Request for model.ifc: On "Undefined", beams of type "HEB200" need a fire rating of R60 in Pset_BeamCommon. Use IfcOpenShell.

First a look at what the model holds.

```python
import ifcopenshell
import ifcopenshell.util.element

model = ifcopenshell.open("model.ifc")
print(model.schema)
storey = next(s for s in model.by_type("IfcBuildingStorey") if s.Name == "Undefined")
beams = [e for e in ifcopenshell.util.element.get_decomposition(storey) if e.is_a("IfcBeam")]
seen = {}
for e in beams:
    element_type = ifcopenshell.util.element.get_type(e)
    key = (element_type.Name if element_type != e and element_type else None, ifcopenshell.util.element.get_pset(e, "Pset_BeamCommon", "FireRating"))
    seen[key] = seen.get(key, 0) + 1
for (name, value), count in sorted(seen.items(), key=str):
    print(count, "x", name, "|", value)
```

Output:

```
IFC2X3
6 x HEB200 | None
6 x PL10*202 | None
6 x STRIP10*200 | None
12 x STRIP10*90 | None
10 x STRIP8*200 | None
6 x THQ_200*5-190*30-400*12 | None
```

```python
import ifcopenshell
import ifcopenshell.api.pset
import ifcopenshell.util.element

model = ifcopenshell.open("model.ifc")

storey = next(s for s in model.by_type("IfcBuildingStorey") if s.Name == "Undefined")
beams = [e for e in ifcopenshell.util.element.get_decomposition(storey) if e.is_a("IfcBeam")]

count = 0
for e in beams:
    element_type = ifcopenshell.util.element.get_type(e)
    if element_type in (None, e) or element_type.Name != "HEB200":
        continue
    # add_pset returns the element's existing set when there is one.
    pset = ifcopenshell.api.pset.add_pset(model, product=e, name="Pset_BeamCommon")
    ifcopenshell.api.pset.edit_pset(model, pset=pset, properties={"FireRating": "R60"})
    count += 1

print(count, "beams updated")

model.write("model_v2.ifc")
```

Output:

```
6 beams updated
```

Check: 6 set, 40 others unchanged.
